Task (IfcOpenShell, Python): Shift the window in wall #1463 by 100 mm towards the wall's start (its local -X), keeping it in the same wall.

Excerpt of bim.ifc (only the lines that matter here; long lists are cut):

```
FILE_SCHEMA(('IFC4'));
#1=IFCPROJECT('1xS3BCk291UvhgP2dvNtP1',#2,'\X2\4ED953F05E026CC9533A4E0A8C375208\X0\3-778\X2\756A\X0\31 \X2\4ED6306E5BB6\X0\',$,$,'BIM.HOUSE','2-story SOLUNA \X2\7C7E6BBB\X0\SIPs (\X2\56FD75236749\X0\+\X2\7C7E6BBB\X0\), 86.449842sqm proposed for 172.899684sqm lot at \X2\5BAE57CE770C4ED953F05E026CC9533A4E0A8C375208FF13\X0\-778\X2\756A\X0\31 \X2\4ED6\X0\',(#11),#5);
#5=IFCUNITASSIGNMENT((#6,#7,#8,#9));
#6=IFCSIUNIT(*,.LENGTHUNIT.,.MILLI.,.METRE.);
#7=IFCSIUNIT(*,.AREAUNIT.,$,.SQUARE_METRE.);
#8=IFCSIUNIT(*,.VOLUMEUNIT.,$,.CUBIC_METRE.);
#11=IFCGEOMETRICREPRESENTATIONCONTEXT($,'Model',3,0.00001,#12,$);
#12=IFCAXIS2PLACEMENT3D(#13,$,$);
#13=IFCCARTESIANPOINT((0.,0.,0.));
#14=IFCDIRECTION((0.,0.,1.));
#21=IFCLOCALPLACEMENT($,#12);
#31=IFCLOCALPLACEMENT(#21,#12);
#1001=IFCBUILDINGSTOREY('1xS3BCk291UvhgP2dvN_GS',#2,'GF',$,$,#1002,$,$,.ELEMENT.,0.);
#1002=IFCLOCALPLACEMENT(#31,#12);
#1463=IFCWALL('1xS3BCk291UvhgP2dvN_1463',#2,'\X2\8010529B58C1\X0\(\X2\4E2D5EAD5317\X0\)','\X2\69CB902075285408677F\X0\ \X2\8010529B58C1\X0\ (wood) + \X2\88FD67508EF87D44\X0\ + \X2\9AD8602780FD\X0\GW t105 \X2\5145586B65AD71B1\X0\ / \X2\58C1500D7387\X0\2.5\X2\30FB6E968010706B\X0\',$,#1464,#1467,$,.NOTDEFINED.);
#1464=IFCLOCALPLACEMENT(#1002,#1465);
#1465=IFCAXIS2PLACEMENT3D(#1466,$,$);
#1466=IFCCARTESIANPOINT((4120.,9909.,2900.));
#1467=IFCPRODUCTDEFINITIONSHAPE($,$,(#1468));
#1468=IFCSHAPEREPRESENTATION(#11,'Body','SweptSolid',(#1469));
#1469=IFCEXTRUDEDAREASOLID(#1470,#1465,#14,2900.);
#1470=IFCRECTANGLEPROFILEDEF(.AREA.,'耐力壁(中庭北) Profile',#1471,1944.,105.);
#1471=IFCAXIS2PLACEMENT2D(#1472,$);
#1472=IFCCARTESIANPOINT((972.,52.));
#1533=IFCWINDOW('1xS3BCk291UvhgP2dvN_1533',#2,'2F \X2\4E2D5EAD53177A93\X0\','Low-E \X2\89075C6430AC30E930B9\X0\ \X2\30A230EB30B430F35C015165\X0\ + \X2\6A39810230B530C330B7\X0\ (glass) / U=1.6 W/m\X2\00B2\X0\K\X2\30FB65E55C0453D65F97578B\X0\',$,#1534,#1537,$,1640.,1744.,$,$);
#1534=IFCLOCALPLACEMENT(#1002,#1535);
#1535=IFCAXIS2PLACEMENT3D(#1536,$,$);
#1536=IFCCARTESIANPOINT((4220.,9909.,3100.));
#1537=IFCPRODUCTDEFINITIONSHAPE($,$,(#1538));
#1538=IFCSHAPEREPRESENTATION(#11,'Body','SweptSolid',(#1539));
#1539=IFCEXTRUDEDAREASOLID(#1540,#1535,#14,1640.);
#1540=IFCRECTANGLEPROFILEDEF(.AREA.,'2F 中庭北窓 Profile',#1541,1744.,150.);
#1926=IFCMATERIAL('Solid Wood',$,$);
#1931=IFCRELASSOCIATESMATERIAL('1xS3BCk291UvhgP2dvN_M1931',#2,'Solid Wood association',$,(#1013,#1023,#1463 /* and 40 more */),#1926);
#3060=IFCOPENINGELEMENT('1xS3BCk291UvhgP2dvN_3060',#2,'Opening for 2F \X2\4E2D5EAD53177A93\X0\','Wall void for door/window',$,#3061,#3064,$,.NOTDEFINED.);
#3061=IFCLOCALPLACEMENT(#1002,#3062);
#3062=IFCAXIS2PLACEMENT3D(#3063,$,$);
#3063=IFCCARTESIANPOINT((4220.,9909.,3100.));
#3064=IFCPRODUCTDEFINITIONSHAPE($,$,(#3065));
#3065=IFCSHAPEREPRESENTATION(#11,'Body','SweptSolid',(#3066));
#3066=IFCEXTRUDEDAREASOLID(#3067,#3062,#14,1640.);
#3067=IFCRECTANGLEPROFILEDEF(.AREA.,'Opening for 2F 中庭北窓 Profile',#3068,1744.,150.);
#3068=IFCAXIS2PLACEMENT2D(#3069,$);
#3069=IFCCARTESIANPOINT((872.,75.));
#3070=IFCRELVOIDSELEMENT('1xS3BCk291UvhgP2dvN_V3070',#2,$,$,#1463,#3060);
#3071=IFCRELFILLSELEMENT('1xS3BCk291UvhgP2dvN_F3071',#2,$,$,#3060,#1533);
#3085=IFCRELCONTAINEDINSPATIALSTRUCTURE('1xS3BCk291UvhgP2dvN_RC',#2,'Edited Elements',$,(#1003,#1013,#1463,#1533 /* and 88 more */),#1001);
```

```python
import ifcopenshell
import ifcopenshell.api.geometry
import ifcopenshell.util.placement

model = ifcopenshell.open("bim.ifc")

window = model.by_guid("1xS3BCk291UvhgP2dvN_1533")
opening = window.FillsVoids[0].RelatingOpeningElement
wall = opening.VoidsElements[0].RelatingBuildingElement

wall_matrix = ifcopenshell.util.placement.get_local_placement(wall.ObjectPlacement)
shift = wall_matrix[:3, 0] * -100.0
before = ifcopenshell.util.placement.get_local_placement(window.ObjectPlacement)[:3, 3].copy()

# The window is not placed relative to its opening, so move both.
for product in (opening, window):
    matrix = ifcopenshell.util.placement.get_local_placement(product.ObjectPlacement)
    matrix[:3, 3] += shift
    ifcopenshell.api.geometry.edit_object_placement(model, product=product, matrix=matrix, is_si=False)

after = ifcopenshell.util.placement.get_local_placement(window.ObjectPlacement)[:3, 3]
print("window moved by", (after - before).round(3) + 0.0)

model.write("bim_updated.ifc")
```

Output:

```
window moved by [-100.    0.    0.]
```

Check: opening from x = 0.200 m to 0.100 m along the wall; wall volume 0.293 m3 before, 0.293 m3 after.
